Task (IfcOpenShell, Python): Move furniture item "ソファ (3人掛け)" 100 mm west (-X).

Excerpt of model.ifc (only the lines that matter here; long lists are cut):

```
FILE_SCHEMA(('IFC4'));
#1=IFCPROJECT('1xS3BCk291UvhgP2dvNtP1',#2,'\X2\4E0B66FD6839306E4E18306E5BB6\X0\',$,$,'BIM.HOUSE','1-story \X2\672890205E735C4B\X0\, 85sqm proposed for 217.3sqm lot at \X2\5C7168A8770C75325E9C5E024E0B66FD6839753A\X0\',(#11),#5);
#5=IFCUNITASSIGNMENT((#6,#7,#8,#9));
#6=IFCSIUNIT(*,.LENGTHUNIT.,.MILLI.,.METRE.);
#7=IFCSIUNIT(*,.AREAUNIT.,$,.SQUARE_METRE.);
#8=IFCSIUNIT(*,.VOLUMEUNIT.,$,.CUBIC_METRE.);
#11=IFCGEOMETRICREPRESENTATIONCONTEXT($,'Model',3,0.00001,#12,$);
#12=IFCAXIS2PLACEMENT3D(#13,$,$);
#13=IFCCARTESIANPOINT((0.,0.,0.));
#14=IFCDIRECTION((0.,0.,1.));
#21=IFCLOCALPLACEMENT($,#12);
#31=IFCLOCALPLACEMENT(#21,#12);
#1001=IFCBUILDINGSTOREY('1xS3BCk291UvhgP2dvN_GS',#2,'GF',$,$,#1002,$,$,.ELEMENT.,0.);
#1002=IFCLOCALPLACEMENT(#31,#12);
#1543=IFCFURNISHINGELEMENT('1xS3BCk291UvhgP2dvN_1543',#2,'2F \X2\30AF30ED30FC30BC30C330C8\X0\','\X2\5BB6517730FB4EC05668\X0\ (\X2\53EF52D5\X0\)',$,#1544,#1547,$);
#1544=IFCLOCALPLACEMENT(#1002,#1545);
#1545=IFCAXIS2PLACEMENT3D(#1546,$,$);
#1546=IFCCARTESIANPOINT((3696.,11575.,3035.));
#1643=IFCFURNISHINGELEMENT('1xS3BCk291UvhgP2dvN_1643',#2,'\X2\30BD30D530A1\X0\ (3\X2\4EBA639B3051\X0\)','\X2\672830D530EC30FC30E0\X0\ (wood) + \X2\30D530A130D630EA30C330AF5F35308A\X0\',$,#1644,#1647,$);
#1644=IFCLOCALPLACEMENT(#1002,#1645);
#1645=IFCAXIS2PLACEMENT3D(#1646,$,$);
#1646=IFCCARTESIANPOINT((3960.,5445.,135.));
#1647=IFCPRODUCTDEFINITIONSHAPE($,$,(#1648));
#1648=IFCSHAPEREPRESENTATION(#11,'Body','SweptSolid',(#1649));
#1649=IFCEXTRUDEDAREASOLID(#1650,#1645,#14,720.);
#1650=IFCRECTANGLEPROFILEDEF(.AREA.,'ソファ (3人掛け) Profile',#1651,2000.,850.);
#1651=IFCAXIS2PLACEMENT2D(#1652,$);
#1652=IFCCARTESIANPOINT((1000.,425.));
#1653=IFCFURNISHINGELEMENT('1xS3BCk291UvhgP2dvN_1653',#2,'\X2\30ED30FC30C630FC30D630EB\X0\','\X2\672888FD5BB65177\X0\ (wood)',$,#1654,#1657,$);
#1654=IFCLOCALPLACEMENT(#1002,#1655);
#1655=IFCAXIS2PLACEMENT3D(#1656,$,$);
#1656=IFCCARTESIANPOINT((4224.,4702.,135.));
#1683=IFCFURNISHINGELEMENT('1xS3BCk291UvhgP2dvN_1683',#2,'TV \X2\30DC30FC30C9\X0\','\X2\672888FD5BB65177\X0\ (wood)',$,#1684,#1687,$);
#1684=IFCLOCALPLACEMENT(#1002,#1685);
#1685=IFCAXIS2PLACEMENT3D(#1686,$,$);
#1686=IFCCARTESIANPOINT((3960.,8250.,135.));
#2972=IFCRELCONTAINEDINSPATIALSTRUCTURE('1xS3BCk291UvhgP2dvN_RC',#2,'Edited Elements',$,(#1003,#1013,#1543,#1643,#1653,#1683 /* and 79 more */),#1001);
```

```python
import ifcopenshell
import ifcopenshell.api.geometry
import ifcopenshell.util.placement
import ifcopenshell.util.unit

model = ifcopenshell.open("model.ifc")
unit_scale = ifcopenshell.util.unit.calculate_unit_scale(model)

item = model.by_guid("1xS3BCk291UvhgP2dvN_1643")
matrix = ifcopenshell.util.placement.get_local_placement(item.ObjectPlacement)
matrix[0, 3] -= 0.1 / unit_scale
ifcopenshell.api.geometry.edit_object_placement(model, product=item, matrix=matrix, is_si=False)

print(ifcopenshell.util.placement.get_local_placement(item.ObjectPlacement).round(3) + 0.0)

model.write("model_updated.ifc")
```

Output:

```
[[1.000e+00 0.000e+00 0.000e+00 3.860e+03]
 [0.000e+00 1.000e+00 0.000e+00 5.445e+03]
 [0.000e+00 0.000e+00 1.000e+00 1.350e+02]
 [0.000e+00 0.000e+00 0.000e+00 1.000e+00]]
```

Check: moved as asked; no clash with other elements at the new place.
